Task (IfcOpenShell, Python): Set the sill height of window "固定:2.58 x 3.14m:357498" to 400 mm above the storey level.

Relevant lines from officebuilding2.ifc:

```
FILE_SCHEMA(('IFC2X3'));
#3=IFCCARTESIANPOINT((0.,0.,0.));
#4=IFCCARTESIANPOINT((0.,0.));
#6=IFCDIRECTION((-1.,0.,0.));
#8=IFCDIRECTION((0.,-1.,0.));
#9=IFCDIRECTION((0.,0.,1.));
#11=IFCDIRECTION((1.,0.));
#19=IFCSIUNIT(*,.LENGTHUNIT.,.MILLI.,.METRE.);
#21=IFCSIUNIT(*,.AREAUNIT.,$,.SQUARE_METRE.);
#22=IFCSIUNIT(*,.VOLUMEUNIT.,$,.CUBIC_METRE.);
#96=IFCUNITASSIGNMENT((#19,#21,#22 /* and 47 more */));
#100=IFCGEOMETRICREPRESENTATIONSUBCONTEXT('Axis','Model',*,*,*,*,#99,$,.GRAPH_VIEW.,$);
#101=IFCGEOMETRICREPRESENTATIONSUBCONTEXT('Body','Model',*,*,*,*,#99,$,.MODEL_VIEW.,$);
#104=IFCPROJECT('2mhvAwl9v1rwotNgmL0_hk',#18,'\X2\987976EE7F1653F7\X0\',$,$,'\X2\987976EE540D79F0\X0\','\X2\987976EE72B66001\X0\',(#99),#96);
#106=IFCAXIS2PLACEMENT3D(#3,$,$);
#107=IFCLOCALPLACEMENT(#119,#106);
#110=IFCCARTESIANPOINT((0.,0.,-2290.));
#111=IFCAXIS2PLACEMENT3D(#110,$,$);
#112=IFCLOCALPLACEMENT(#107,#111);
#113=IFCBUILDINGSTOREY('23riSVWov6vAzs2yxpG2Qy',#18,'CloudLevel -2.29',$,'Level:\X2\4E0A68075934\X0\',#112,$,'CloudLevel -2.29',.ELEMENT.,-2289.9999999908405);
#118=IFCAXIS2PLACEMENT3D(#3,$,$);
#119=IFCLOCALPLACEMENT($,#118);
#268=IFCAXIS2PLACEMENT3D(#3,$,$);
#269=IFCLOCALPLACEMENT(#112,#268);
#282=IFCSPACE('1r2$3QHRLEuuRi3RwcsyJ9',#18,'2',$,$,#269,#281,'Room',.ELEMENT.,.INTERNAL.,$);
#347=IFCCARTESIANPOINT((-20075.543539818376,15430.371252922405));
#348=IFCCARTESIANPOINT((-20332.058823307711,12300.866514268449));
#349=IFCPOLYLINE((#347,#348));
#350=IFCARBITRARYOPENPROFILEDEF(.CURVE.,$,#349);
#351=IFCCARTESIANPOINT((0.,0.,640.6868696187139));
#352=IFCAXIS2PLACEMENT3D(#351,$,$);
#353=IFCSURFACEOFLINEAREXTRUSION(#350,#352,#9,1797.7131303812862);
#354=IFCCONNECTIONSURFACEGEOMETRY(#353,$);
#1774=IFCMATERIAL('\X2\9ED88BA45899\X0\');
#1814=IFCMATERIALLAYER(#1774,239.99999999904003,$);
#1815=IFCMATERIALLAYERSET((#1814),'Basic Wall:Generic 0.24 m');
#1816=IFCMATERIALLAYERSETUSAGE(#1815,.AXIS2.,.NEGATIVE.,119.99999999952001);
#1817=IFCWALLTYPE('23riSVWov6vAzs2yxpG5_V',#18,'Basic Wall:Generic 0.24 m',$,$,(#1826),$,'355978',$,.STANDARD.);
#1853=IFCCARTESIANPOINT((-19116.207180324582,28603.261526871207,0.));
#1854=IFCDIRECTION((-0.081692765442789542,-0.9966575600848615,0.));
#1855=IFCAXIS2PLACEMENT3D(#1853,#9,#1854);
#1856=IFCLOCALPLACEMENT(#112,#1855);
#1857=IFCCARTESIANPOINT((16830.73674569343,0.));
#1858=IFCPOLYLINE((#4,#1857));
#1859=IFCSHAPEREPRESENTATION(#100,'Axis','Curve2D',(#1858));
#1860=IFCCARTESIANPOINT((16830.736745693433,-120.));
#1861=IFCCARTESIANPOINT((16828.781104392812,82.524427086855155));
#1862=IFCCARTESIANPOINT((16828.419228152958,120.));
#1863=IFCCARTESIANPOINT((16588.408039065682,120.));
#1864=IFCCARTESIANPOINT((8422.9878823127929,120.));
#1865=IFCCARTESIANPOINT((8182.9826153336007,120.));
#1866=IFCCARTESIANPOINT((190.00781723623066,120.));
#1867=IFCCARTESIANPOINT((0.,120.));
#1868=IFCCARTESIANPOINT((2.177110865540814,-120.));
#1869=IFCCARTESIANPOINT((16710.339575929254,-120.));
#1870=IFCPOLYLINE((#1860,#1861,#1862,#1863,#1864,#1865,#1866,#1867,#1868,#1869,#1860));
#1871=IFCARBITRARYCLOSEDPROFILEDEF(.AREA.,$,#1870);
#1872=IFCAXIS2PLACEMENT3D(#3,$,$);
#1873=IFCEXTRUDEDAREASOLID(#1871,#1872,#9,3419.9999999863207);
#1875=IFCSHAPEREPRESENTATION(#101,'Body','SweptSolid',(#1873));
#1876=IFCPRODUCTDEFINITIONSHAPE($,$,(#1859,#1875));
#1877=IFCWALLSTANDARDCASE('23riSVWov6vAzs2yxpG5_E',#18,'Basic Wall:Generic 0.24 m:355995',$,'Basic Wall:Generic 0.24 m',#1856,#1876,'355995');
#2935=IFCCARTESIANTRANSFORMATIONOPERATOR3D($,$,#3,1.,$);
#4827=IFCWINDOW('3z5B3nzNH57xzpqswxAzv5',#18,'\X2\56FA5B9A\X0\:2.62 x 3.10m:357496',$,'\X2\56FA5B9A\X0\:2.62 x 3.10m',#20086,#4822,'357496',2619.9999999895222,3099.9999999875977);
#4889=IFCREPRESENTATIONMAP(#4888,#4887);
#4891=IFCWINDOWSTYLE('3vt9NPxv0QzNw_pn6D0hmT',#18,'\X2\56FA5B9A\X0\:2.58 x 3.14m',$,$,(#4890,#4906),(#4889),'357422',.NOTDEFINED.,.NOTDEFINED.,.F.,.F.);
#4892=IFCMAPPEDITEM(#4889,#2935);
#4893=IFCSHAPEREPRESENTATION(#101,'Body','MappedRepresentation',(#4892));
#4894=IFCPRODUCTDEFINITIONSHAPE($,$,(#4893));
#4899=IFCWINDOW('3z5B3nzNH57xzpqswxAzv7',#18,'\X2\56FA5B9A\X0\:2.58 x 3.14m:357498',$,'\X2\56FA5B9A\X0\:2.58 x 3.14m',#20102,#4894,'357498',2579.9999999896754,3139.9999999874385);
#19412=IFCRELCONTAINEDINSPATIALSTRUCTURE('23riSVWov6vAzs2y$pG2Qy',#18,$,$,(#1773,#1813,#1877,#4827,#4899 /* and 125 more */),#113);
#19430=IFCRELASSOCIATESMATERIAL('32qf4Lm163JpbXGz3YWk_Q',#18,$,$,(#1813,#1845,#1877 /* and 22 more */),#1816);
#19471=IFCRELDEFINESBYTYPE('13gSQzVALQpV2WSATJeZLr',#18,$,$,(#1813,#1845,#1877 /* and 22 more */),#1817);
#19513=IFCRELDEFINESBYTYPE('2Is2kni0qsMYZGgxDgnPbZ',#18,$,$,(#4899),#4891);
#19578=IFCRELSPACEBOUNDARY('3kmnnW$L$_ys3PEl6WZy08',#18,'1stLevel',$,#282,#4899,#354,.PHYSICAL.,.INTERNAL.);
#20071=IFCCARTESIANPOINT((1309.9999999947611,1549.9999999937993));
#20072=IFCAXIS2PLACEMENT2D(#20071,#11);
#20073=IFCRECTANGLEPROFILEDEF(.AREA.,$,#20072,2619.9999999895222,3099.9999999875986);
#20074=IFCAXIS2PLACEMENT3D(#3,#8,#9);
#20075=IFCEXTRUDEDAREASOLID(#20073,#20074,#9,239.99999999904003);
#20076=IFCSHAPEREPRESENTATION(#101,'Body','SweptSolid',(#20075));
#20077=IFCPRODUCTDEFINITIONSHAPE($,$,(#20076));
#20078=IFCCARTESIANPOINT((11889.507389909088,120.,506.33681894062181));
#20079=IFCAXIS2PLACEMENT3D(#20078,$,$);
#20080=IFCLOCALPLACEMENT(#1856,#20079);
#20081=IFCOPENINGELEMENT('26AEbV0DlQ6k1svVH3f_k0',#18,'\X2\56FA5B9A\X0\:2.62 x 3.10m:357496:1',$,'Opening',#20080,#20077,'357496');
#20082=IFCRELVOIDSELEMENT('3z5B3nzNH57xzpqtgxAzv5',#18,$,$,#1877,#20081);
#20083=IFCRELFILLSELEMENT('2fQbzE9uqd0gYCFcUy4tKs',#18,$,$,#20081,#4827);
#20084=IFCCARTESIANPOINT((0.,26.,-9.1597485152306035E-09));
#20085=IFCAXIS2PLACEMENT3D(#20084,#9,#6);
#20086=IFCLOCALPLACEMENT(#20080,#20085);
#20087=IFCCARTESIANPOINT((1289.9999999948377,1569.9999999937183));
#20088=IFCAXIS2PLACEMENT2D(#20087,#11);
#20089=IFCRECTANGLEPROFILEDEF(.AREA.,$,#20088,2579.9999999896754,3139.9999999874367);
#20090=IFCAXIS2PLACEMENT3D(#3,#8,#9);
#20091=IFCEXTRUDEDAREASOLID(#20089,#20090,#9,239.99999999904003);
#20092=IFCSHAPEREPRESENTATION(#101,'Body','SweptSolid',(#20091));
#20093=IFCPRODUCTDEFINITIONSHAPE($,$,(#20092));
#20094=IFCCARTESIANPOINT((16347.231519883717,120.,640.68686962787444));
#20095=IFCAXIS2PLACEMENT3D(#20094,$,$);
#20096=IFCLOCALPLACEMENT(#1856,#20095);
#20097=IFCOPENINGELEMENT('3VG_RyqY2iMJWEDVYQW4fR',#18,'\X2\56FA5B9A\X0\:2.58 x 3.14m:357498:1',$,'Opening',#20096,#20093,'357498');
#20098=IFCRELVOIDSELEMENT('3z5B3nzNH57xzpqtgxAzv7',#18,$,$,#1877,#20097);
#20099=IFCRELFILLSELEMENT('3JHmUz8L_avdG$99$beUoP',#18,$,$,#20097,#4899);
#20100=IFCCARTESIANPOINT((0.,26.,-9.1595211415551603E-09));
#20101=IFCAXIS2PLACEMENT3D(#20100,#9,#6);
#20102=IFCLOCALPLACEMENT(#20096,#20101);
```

```python
import numpy as np
import ifcopenshell
import ifcopenshell.api.geometry
import ifcopenshell.geom
import ifcopenshell.util.element
import ifcopenshell.util.placement
import ifcopenshell.util.shape
import ifcopenshell.util.unit

model = ifcopenshell.open("officebuilding2.ifc")
unit_scale = ifcopenshell.util.unit.calculate_unit_scale(model)

window = model.by_guid("3z5B3nzNH57xzpqswxAzv7")
opening = window.FillsVoids[0].RelatingOpeningElement
storey = ifcopenshell.util.element.get_container(window, ifc_class="IfcBuildingStorey")
level = ifcopenshell.util.placement.get_local_placement(storey.ObjectPlacement)[2, 3]

# The opening's origin need not be at the sill, so measure its lowest point.
shape = ifcopenshell.geom.create_shape(ifcopenshell.geom.settings(), opening)
bottom = ifcopenshell.util.shape.get_shape_bottom_elevation(shape, shape.geometry) / unit_scale
dz = level + 0.4 / unit_scale - bottom

shift = np.array([0.0, 0.0, dz])
# The window is placed relative to its opening, so it follows when the opening moves.
matrix = ifcopenshell.util.placement.get_local_placement(opening.ObjectPlacement)
matrix[:3, 3] += shift
ifcopenshell.api.geometry.edit_object_placement(
    model, product=opening, matrix=matrix, is_si=False, should_transform_children=True
)

# Space boundary surfaces are stored in each space's coordinates; move them too.
for rel in window.ProvidesBoundaries:
    if not rel.ConnectionGeometry:
        continue
    surface = rel.ConnectionGeometry.SurfaceOnRelatingElement
    space_matrix = ifcopenshell.util.placement.get_local_placement(rel.RelatingSpace.ObjectPlacement)
    point = np.array(surface.Position.Location.Coordinates) + space_matrix[:3, :3].T @ shift
    surface.Position = model.createIfcAxis2Placement3D(
        model.createIfcCartesianPoint(point.tolist()), surface.Position.Axis, surface.Position.RefDirection
    )

print(f"moved by {dz * unit_scale:+.3f} m")

model.write("officebuilding2_edited.ifc")
```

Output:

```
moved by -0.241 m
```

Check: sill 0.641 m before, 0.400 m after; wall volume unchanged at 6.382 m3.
